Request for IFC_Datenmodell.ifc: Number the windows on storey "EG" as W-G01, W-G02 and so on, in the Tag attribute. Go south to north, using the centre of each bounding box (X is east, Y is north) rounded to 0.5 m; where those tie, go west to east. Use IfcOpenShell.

First a look at what the model holds.

```python
import ifcopenshell
import ifcopenshell.util.element
import ifcopenshell.util.placement

model = ifcopenshell.open("IFC_Datenmodell.ifc")
print(model.schema)
storey = next(s for s in model.by_type("IfcBuildingStorey") if s.Name == "EG")
windows = [e for e in ifcopenshell.util.element.get_decomposition(storey) if e.is_a("IfcWindow")]
for e in sorted(windows, key=lambda e: e.id()):
    origin = ifcopenshell.util.placement.get_local_placement(e.ObjectPlacement)[:3, 3]
    print(e.id(), e.Tag, e.Name, origin.round(2) + 0.0, sep=" | ")
```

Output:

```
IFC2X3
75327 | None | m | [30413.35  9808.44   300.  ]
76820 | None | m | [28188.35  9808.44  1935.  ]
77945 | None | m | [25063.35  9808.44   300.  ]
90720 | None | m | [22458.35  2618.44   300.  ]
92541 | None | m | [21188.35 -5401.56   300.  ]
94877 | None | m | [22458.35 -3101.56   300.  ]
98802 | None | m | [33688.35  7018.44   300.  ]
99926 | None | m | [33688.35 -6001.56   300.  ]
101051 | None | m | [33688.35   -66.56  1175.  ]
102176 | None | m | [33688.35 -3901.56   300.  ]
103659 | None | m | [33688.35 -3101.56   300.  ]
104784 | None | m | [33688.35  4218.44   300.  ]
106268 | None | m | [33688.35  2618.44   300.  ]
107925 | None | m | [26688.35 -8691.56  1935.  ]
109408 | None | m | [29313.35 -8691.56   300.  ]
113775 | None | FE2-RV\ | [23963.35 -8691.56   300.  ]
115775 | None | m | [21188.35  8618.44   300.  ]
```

```python
import ifcopenshell
import ifcopenshell.geom
import ifcopenshell.util.element
import ifcopenshell.util.shape

model = ifcopenshell.open("IFC_Datenmodell.ifc")
settings = ifcopenshell.geom.settings()
settings.set("use-world-coords", True)


def centre(element):
    shape = ifcopenshell.geom.create_shape(settings, element)
    return ifcopenshell.util.shape.get_bbox_centroid(shape.geometry)


storey = next(s for s in model.by_type("IfcBuildingStorey") if s.Name == "EG")
windows = [e for e in ifcopenshell.util.element.get_decomposition(storey) if e.is_a("IfcWindow")]

# Insertion points can sit at a corner or the storey origin, so sort by the geometry (in metres).
centres = {e: centre(e) for e in windows}
windows.sort(key=lambda e: (round(centres[e][1] / 0.5), centres[e][0]))

for i, e in enumerate(windows, start=1):
    number = f"W-G{i:02d}"
    e.Tag = number
    print(e.id(), number)

model.write("IFC_Datenmodell_rev.ifc")
```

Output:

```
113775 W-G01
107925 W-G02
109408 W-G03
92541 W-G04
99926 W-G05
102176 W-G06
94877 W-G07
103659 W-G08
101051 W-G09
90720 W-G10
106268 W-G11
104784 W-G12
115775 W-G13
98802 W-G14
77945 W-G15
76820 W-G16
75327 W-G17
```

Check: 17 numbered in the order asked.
